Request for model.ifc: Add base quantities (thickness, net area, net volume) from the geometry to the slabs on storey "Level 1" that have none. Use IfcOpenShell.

First a look at what the model holds.

```python
import ifcopenshell
import ifcopenshell.util.element
import ifcopenshell.util.unit

model = ifcopenshell.open("model.ifc")
print(model.schema)
for unit_type in ("LENGTHUNIT", "AREAUNIT", "VOLUMEUNIT"):
    print(unit_type, ifcopenshell.util.unit.calculate_unit_scale(model, unit_type))
storey = next(s for s in model.by_type("IfcBuildingStorey") if s.Name == "Level 1")
slabs = [e for e in ifcopenshell.util.element.get_decomposition(storey) if e.is_a("IfcSlab")]
for e in sorted(slabs, key=lambda e: e.id()):
    print(e.id(), e.is_a(), e.Name, list(ifcopenshell.util.element.get_psets(e, qtos_only=True)), sep=" | ")
```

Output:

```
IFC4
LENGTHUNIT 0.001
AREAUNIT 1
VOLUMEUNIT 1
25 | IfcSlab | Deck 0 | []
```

```python
import ifcopenshell
import ifcopenshell.api.pset
import ifcopenshell.geom
import ifcopenshell.util.element
import ifcopenshell.util.shape
import ifcopenshell.util.unit

model = ifcopenshell.open("model.ifc")
unit_scale = ifcopenshell.util.unit.calculate_unit_scale(model)
area_scale = ifcopenshell.util.unit.calculate_unit_scale(model, "AREAUNIT")
volume_scale = ifcopenshell.util.unit.calculate_unit_scale(model, "VOLUMEUNIT")
settings = ifcopenshell.geom.settings()

storey = next(s for s in model.by_type("IfcBuildingStorey") if s.Name == "Level 1")
slabs = [e for e in ifcopenshell.util.element.get_decomposition(storey) if e.is_a("IfcSlab")]

for e in sorted(slabs, key=lambda e: e.id()):
    if ifcopenshell.util.element.get_psets(e, qtos_only=True, should_inherit=False):
        continue
    # Geometry comes back in metres, in the element's own axes.
    shape = ifcopenshell.geom.create_shape(settings, e)
    values = {
        "Width": ifcopenshell.util.shape.get_z(shape.geometry) / unit_scale,
        "NetArea": ifcopenshell.util.shape.get_footprint_area(shape.geometry) / area_scale,
        "NetVolume": ifcopenshell.util.shape.get_volume(shape.geometry) / volume_scale,
    }
    qto = ifcopenshell.api.pset.add_qto(model, product=e, name="Qto_SlabBaseQuantities")
    ifcopenshell.api.pset.edit_qto(model, qto=qto, properties=values)
    print(e.id(), {k: round(v, 3) for k, v in values.items()})

model.write("model_updated.ifc")
```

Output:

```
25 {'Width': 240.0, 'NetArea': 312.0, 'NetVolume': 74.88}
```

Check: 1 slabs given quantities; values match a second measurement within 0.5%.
